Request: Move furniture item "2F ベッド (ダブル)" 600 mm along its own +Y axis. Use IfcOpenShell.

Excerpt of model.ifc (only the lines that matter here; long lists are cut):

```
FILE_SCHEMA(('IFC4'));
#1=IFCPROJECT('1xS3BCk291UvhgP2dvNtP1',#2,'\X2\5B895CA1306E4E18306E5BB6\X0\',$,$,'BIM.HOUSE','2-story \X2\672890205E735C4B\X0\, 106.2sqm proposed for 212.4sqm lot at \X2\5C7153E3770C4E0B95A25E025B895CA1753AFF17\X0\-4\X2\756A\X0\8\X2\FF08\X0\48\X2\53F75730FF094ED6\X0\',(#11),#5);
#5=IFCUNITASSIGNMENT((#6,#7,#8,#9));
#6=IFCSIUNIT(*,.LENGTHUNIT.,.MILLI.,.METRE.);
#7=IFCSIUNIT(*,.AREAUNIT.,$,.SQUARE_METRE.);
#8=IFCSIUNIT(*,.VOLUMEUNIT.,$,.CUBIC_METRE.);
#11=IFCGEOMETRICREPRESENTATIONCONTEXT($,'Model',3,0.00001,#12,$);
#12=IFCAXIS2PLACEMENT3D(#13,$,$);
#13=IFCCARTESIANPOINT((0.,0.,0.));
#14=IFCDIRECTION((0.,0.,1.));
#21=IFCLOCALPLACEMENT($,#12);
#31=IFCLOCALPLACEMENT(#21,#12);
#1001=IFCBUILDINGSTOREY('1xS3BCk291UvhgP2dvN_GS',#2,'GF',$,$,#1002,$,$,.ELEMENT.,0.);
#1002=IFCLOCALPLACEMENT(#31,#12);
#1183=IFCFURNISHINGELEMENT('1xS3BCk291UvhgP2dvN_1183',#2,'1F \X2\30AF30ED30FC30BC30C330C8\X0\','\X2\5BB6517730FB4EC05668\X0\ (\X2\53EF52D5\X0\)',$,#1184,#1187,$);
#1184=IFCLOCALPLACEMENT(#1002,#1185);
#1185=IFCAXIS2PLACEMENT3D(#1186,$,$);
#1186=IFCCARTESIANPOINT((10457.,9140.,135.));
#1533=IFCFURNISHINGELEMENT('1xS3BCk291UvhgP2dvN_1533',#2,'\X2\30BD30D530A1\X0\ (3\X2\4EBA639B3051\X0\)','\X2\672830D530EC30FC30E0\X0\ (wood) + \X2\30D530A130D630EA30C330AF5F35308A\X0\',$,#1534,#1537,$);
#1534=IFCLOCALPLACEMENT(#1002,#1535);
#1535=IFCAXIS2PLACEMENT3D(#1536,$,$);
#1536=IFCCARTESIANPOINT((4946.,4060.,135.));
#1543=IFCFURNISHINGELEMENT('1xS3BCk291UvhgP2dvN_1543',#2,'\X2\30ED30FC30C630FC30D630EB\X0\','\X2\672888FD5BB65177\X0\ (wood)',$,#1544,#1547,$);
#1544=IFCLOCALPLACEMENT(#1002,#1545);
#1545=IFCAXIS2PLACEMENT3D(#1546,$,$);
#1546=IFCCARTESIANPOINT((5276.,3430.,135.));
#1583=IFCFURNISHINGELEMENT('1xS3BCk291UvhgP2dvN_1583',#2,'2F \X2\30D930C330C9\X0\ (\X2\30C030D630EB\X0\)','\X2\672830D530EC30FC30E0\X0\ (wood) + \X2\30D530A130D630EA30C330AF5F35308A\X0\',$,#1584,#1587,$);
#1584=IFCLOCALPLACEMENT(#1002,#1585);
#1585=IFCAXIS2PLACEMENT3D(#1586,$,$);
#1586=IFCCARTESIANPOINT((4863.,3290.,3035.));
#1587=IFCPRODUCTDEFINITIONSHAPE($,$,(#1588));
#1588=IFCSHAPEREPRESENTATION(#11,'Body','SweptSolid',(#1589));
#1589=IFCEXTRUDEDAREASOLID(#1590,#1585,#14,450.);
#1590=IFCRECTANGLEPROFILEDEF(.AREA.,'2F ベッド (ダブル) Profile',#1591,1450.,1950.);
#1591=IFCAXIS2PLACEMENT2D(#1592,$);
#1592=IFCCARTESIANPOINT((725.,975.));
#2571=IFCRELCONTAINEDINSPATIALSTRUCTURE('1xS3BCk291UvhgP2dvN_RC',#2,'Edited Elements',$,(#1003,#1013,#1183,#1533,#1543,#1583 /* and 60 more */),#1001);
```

```python
import ifcopenshell
import ifcopenshell.api.geometry
import ifcopenshell.util.placement

model = ifcopenshell.open("model.ifc")

item = model.by_guid("1xS3BCk291UvhgP2dvN_1583")
matrix = ifcopenshell.util.placement.get_local_placement(item.ObjectPlacement)
matrix[:3, 3] += matrix[:3, 1] * 600.0
ifcopenshell.api.geometry.edit_object_placement(model, product=item, matrix=matrix, is_si=False)

print(ifcopenshell.util.placement.get_local_placement(item.ObjectPlacement).round(3) + 0.0)

model.write("model_updated.ifc")
```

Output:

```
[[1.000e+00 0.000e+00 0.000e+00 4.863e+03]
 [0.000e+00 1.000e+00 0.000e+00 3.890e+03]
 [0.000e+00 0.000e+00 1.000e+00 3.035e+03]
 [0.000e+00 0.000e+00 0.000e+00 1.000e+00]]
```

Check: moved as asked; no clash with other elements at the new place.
